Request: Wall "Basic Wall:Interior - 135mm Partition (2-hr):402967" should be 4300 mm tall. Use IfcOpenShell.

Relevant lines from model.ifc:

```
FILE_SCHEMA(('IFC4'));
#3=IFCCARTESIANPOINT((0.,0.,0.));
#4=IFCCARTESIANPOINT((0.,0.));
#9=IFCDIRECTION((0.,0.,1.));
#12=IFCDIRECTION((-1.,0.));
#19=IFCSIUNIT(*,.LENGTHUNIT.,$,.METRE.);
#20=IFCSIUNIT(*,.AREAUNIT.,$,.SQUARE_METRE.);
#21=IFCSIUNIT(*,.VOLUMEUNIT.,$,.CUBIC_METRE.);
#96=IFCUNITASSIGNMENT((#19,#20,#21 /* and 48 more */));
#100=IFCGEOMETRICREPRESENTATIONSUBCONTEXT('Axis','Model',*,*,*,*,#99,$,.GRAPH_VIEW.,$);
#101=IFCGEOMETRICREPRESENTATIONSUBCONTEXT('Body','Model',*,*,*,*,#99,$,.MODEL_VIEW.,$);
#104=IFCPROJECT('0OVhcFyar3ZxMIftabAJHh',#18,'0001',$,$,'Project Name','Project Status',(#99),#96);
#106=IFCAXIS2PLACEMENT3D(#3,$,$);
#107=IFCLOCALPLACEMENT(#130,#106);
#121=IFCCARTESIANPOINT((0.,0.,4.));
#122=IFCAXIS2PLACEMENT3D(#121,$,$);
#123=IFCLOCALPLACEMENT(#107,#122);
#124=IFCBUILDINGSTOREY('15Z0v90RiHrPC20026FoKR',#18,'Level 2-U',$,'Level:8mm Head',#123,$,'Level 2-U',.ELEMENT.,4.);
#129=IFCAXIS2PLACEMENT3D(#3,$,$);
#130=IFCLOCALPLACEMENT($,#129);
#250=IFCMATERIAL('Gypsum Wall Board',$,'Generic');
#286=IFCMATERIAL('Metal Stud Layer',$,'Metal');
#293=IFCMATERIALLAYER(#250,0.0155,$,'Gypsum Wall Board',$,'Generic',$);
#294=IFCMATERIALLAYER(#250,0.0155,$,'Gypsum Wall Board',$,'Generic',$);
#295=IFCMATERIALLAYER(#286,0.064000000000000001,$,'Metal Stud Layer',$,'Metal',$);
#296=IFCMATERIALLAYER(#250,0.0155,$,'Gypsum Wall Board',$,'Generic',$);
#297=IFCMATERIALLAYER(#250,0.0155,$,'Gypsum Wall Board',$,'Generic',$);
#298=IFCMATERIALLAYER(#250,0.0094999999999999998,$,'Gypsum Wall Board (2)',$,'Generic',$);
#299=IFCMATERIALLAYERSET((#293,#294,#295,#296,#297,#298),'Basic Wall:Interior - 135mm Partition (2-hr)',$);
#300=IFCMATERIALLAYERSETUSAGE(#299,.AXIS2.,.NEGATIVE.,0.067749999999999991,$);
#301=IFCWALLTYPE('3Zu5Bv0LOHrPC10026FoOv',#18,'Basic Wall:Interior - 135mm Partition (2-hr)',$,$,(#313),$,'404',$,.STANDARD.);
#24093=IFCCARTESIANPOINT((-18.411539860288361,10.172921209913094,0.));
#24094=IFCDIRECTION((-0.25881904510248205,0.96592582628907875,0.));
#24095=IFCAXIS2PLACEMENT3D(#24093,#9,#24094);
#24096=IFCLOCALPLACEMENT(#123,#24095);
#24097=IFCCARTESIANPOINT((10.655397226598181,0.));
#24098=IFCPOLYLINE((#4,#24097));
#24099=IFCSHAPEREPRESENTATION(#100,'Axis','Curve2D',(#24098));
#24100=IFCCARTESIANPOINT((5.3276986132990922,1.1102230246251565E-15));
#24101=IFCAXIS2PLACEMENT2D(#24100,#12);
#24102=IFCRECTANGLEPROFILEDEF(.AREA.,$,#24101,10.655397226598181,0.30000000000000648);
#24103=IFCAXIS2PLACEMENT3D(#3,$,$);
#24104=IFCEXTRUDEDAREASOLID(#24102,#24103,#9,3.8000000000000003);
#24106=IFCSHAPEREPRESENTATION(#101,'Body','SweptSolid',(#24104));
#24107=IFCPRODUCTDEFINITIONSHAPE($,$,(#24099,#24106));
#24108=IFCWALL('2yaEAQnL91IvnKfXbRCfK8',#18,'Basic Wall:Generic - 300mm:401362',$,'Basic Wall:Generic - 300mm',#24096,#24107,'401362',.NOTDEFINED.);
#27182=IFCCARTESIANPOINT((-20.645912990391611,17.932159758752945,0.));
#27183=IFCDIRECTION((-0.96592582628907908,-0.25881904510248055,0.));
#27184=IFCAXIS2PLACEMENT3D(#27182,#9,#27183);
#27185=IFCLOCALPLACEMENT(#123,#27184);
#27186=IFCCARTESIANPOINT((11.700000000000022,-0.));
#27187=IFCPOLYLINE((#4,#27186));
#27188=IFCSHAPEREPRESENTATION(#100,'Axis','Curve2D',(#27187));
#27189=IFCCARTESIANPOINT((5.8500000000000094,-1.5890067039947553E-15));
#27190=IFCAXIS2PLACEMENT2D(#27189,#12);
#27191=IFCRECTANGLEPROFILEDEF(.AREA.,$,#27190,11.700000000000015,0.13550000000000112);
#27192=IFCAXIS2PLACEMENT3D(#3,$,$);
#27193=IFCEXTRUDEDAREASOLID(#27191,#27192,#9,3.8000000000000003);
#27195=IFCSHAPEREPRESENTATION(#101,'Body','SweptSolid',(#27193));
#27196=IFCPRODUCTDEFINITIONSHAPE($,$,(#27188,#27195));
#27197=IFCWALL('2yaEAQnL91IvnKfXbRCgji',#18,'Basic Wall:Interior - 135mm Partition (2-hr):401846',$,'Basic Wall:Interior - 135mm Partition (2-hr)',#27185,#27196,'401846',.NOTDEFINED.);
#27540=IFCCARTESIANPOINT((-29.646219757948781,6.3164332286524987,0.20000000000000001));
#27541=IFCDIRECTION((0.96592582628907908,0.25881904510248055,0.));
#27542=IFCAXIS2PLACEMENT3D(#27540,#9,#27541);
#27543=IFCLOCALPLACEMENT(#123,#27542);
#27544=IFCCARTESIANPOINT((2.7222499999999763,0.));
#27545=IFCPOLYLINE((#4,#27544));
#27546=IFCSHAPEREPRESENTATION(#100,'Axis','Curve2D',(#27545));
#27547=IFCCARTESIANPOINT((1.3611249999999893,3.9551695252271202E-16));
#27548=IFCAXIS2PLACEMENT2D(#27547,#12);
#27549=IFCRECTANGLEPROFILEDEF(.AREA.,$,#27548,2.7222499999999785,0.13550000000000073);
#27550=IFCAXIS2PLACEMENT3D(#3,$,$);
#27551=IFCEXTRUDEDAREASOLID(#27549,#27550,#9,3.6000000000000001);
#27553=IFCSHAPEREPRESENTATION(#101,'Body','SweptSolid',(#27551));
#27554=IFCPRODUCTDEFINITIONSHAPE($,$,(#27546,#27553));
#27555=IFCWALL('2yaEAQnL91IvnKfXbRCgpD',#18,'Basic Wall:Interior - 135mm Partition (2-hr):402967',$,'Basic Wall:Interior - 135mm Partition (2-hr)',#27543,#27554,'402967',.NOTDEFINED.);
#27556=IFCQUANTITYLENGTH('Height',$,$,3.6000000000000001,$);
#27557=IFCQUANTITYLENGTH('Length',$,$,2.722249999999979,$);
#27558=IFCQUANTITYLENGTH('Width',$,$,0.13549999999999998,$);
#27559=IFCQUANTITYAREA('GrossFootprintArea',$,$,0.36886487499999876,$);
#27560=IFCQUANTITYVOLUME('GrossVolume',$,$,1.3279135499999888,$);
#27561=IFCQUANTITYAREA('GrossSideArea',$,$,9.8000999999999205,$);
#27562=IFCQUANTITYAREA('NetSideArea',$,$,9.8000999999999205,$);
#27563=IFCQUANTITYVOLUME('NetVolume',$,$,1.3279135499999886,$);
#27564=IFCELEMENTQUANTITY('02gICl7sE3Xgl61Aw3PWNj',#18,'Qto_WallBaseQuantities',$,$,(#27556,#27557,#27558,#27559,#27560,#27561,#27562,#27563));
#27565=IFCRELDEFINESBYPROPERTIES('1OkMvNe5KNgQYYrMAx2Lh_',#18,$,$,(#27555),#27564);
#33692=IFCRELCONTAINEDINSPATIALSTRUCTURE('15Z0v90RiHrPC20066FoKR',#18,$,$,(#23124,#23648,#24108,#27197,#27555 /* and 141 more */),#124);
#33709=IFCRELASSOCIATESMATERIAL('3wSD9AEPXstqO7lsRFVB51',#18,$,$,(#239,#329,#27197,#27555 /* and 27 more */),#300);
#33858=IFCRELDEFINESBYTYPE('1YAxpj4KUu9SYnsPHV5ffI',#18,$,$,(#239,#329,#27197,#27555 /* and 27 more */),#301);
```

```python
import ifcopenshell
import ifcopenshell.api.pset
import ifcopenshell.geom
import ifcopenshell.util.element
import ifcopenshell.util.representation
import ifcopenshell.util.shape
import ifcopenshell.util.unit

model = ifcopenshell.open("model.ifc")
unit_scale = ifcopenshell.util.unit.calculate_unit_scale(model)
area_scale = ifcopenshell.util.unit.calculate_unit_scale(model, "AREAUNIT")
volume_scale = ifcopenshell.util.unit.calculate_unit_scale(model, "VOLUMEUNIT")
settings = ifcopenshell.geom.settings()


def volume(element):
    """Net volume in cubic metres, openings subtracted."""
    shape = ifcopenshell.geom.create_shape(settings, element)
    return ifcopenshell.util.shape.get_volume(shape.geometry)


wall = model.by_guid("2yaEAQnL91IvnKfXbRCgpD")
before = volume(wall)

body = ifcopenshell.util.representation.get_representation(wall, "Model", "Body")
solid = body.Items[0]
old_height = solid.Depth
solid.Depth = 4.3
after = volume(wall)
thickness = 0.1355  # wall thickness in metres

# Update the stored height, areas and volumes.
qto = model.by_id(ifcopenshell.util.element.get_pset(wall, "Qto_WallBaseQuantities", should_inherit=False)["id"])
ifcopenshell.api.pset.edit_qto(model, qto=qto, properties={
    "Height": solid.Depth,
    "GrossVolume": ifcopenshell.util.element.get_pset(wall, "Qto_WallBaseQuantities", "GrossVolume") * solid.Depth / old_height,
    "GrossSideArea": ifcopenshell.util.element.get_pset(wall, "Qto_WallBaseQuantities", "GrossSideArea") * solid.Depth / old_height,
    "NetSideArea": after / thickness / area_scale,
    "NetVolume": after / volume_scale,
})

print(f"height {old_height:g} -> {solid.Depth:g}, volume {before:.3f} -> {after:.3f} m3")

model.write("model_v2.ifc")
```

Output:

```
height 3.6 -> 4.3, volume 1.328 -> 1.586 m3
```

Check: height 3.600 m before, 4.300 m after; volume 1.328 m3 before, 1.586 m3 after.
